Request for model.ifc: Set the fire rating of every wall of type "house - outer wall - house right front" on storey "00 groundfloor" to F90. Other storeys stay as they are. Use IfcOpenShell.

First a look at what the model holds.

```python
import ifcopenshell
import ifcopenshell.util.element

model = ifcopenshell.open("model.ifc")
print(model.schema)
storey = next(s for s in model.by_type("IfcBuildingStorey") if s.Name == "00 groundfloor")
walls = [e for e in ifcopenshell.util.element.get_decomposition(storey) if e.is_a("IfcWall")]
seen = {}
for e in walls:
    element_type = ifcopenshell.util.element.get_type(e)
    key = (element_type.Name if element_type != e and element_type else None, ifcopenshell.util.element.get_pset(e, "Pset_WallCommon", "FireRating"))
    seen[key] = seen.get(key, 0) + 1
for (name, value), count in sorted(seen.items(), key=str):
    print(count, "x", name, "|", value)
```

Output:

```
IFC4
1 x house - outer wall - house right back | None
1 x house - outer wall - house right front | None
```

```python
import ifcopenshell
import ifcopenshell.api.pset
import ifcopenshell.util.element

model = ifcopenshell.open("model.ifc")

storey = next(s for s in model.by_type("IfcBuildingStorey") if s.Name == "00 groundfloor")
walls = [e for e in ifcopenshell.util.element.get_decomposition(storey) if e.is_a("IfcWall")]

count = 0
for e in walls:
    element_type = ifcopenshell.util.element.get_type(e)
    if element_type in (None, e) or element_type.Name != "house - outer wall - house right front":
        continue
    # add_pset returns the element's existing set when there is one.
    pset = ifcopenshell.api.pset.add_pset(model, product=e, name="Pset_WallCommon")
    ifcopenshell.api.pset.edit_pset(model, pset=pset, properties={"FireRating": "F90"})
    count += 1

print(count, "walls updated")

model.write("model_rev.ifc")
```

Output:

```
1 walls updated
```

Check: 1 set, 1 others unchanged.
